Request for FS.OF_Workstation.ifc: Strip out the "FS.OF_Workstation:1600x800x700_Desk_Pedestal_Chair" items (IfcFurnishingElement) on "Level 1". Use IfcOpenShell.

First a look at what the model holds.

```python
import ifcopenshell
import ifcopenshell.util.element

model = ifcopenshell.open("FS.OF_Workstation.ifc")
print(model.schema)
storey = next(s for s in model.by_type("IfcBuildingStorey") if s.Name == "Level 1")
furniture = [e for e in ifcopenshell.util.element.get_decomposition(storey) if e.is_a("IfcFurnishingElement")]
seen = {}
for e in furniture:
    element_type = ifcopenshell.util.element.get_type(e)
    name = element_type.Name if element_type not in (None, e) else None
    seen[name] = seen.get(name, 0) + 1
for name, count in sorted(seen.items(), key=str):
    print(count, "x", name)
```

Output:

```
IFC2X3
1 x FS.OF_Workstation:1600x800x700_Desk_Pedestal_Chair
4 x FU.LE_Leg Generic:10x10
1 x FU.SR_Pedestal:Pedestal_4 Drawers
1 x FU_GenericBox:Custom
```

```python
import ifcopenshell
import ifcopenshell.api.root
import ifcopenshell.util.element

model = ifcopenshell.open("FS.OF_Workstation.ifc")

storey = next(s for s in model.by_type("IfcBuildingStorey") if s.Name == "Level 1")
furniture = [e for e in ifcopenshell.util.element.get_decomposition(storey) if e.is_a("IfcFurnishingElement")]
targets = [e for e in furniture if (t := ifcopenshell.util.element.get_type(e)) not in (None, e) and t.Name == "FS.OF_Workstation:1600x800x700_Desk_Pedestal_Chair"]

for e in targets:
    ifcopenshell.api.root.remove_product(model, product=e)
print(len(targets), "removed")

model.write("FS.OF_Workstation_v2.ifc")
```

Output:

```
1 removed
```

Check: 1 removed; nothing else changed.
